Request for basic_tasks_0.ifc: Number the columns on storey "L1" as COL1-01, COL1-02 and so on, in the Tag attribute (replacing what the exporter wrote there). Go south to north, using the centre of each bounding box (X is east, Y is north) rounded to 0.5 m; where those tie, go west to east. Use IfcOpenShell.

First a look at what the model holds.

```python
import ifcopenshell
import ifcopenshell.util.element
import ifcopenshell.util.placement

model = ifcopenshell.open("basic_tasks_0.ifc")
print(model.schema)
storey = next(s for s in model.by_type("IfcBuildingStorey") if s.Name == "L1")
columns = [e for e in ifcopenshell.util.element.get_decomposition(storey) if e.is_a("IfcColumn")]
for e in sorted(columns, key=lambda e: e.id()):
    origin = ifcopenshell.util.placement.get_local_placement(e.ObjectPlacement)[:3, 3]
    print(e.id(), e.Tag, e.Name, origin.round(2) + 0.0, sep=" | ")
```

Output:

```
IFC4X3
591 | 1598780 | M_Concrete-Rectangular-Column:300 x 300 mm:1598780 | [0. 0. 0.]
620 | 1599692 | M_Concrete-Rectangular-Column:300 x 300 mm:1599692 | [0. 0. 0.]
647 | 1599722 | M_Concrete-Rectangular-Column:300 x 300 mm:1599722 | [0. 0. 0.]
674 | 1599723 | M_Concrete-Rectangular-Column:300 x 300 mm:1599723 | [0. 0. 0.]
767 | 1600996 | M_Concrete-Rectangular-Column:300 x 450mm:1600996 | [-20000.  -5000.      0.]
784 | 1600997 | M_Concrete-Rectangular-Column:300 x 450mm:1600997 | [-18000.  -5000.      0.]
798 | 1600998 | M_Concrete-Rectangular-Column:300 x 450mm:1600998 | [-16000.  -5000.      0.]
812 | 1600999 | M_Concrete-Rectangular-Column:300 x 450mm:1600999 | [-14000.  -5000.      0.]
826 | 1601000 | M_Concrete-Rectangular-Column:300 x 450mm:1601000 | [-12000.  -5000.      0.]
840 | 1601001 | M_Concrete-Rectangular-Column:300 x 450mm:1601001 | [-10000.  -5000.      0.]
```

```python
import ifcopenshell
import ifcopenshell.geom
import ifcopenshell.util.element
import ifcopenshell.util.shape

model = ifcopenshell.open("basic_tasks_0.ifc")
settings = ifcopenshell.geom.settings()
settings.set("use-world-coords", True)


def centre(element):
    shape = ifcopenshell.geom.create_shape(settings, element)
    return ifcopenshell.util.shape.get_bbox_centroid(shape.geometry)


storey = next(s for s in model.by_type("IfcBuildingStorey") if s.Name == "L1")
columns = [e for e in ifcopenshell.util.element.get_decomposition(storey) if e.is_a("IfcColumn")]

# Insertion points can sit at a corner or the storey origin, so sort by the geometry (in metres).
centres = {e: centre(e) for e in columns}
columns.sort(key=lambda e: (round(centres[e][1] / 0.5), centres[e][0]))

for i, e in enumerate(columns, start=1):
    number = f"COL1-{i:02d}"
    e.Tag = number
    print(e.id(), number)

model.write("basic_tasks_0_v2.ifc")
```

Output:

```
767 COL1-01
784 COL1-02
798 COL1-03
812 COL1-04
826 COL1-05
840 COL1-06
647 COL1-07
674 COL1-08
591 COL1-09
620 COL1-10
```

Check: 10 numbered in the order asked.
